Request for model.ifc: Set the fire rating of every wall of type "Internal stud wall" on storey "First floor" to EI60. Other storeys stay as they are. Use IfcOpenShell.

First a look at what the model holds.

```python
import ifcopenshell
import ifcopenshell.util.element

model = ifcopenshell.open("model.ifc")
print(model.schema)
storey = next(s for s in model.by_type("IfcBuildingStorey") if s.Name == "First floor")
walls = [e for e in ifcopenshell.util.element.get_decomposition(storey) if e.is_a("IfcWall")]
seen = {}
for e in walls:
    element_type = ifcopenshell.util.element.get_type(e)
    key = (element_type.Name if element_type != e and element_type else None, ifcopenshell.util.element.get_pset(e, "Pset_WallCommon", "FireRating"))
    seen[key] = seen.get(key, 0) + 1
for (name, value), count in sorted(seen.items(), key=str):
    print(count, "x", name, "|", value)
```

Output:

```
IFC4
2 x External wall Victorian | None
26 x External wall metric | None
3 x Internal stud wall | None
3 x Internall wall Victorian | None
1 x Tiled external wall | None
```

```python
import ifcopenshell
import ifcopenshell.api.pset
import ifcopenshell.util.element

model = ifcopenshell.open("model.ifc")

storey = next(s for s in model.by_type("IfcBuildingStorey") if s.Name == "First floor")
walls = [e for e in ifcopenshell.util.element.get_decomposition(storey) if e.is_a("IfcWall")]

count = 0
for e in walls:
    element_type = ifcopenshell.util.element.get_type(e)
    if element_type in (None, e) or element_type.Name != "Internal stud wall":
        continue
    # add_pset returns the element's existing set when there is one.
    pset = ifcopenshell.api.pset.add_pset(model, product=e, name="Pset_WallCommon")
    ifcopenshell.api.pset.edit_pset(model, pset=pset, properties={"FireRating": "EI60"})
    count += 1

print(count, "walls updated")

model.write("model_updated.ifc")
```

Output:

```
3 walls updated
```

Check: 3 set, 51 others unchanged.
